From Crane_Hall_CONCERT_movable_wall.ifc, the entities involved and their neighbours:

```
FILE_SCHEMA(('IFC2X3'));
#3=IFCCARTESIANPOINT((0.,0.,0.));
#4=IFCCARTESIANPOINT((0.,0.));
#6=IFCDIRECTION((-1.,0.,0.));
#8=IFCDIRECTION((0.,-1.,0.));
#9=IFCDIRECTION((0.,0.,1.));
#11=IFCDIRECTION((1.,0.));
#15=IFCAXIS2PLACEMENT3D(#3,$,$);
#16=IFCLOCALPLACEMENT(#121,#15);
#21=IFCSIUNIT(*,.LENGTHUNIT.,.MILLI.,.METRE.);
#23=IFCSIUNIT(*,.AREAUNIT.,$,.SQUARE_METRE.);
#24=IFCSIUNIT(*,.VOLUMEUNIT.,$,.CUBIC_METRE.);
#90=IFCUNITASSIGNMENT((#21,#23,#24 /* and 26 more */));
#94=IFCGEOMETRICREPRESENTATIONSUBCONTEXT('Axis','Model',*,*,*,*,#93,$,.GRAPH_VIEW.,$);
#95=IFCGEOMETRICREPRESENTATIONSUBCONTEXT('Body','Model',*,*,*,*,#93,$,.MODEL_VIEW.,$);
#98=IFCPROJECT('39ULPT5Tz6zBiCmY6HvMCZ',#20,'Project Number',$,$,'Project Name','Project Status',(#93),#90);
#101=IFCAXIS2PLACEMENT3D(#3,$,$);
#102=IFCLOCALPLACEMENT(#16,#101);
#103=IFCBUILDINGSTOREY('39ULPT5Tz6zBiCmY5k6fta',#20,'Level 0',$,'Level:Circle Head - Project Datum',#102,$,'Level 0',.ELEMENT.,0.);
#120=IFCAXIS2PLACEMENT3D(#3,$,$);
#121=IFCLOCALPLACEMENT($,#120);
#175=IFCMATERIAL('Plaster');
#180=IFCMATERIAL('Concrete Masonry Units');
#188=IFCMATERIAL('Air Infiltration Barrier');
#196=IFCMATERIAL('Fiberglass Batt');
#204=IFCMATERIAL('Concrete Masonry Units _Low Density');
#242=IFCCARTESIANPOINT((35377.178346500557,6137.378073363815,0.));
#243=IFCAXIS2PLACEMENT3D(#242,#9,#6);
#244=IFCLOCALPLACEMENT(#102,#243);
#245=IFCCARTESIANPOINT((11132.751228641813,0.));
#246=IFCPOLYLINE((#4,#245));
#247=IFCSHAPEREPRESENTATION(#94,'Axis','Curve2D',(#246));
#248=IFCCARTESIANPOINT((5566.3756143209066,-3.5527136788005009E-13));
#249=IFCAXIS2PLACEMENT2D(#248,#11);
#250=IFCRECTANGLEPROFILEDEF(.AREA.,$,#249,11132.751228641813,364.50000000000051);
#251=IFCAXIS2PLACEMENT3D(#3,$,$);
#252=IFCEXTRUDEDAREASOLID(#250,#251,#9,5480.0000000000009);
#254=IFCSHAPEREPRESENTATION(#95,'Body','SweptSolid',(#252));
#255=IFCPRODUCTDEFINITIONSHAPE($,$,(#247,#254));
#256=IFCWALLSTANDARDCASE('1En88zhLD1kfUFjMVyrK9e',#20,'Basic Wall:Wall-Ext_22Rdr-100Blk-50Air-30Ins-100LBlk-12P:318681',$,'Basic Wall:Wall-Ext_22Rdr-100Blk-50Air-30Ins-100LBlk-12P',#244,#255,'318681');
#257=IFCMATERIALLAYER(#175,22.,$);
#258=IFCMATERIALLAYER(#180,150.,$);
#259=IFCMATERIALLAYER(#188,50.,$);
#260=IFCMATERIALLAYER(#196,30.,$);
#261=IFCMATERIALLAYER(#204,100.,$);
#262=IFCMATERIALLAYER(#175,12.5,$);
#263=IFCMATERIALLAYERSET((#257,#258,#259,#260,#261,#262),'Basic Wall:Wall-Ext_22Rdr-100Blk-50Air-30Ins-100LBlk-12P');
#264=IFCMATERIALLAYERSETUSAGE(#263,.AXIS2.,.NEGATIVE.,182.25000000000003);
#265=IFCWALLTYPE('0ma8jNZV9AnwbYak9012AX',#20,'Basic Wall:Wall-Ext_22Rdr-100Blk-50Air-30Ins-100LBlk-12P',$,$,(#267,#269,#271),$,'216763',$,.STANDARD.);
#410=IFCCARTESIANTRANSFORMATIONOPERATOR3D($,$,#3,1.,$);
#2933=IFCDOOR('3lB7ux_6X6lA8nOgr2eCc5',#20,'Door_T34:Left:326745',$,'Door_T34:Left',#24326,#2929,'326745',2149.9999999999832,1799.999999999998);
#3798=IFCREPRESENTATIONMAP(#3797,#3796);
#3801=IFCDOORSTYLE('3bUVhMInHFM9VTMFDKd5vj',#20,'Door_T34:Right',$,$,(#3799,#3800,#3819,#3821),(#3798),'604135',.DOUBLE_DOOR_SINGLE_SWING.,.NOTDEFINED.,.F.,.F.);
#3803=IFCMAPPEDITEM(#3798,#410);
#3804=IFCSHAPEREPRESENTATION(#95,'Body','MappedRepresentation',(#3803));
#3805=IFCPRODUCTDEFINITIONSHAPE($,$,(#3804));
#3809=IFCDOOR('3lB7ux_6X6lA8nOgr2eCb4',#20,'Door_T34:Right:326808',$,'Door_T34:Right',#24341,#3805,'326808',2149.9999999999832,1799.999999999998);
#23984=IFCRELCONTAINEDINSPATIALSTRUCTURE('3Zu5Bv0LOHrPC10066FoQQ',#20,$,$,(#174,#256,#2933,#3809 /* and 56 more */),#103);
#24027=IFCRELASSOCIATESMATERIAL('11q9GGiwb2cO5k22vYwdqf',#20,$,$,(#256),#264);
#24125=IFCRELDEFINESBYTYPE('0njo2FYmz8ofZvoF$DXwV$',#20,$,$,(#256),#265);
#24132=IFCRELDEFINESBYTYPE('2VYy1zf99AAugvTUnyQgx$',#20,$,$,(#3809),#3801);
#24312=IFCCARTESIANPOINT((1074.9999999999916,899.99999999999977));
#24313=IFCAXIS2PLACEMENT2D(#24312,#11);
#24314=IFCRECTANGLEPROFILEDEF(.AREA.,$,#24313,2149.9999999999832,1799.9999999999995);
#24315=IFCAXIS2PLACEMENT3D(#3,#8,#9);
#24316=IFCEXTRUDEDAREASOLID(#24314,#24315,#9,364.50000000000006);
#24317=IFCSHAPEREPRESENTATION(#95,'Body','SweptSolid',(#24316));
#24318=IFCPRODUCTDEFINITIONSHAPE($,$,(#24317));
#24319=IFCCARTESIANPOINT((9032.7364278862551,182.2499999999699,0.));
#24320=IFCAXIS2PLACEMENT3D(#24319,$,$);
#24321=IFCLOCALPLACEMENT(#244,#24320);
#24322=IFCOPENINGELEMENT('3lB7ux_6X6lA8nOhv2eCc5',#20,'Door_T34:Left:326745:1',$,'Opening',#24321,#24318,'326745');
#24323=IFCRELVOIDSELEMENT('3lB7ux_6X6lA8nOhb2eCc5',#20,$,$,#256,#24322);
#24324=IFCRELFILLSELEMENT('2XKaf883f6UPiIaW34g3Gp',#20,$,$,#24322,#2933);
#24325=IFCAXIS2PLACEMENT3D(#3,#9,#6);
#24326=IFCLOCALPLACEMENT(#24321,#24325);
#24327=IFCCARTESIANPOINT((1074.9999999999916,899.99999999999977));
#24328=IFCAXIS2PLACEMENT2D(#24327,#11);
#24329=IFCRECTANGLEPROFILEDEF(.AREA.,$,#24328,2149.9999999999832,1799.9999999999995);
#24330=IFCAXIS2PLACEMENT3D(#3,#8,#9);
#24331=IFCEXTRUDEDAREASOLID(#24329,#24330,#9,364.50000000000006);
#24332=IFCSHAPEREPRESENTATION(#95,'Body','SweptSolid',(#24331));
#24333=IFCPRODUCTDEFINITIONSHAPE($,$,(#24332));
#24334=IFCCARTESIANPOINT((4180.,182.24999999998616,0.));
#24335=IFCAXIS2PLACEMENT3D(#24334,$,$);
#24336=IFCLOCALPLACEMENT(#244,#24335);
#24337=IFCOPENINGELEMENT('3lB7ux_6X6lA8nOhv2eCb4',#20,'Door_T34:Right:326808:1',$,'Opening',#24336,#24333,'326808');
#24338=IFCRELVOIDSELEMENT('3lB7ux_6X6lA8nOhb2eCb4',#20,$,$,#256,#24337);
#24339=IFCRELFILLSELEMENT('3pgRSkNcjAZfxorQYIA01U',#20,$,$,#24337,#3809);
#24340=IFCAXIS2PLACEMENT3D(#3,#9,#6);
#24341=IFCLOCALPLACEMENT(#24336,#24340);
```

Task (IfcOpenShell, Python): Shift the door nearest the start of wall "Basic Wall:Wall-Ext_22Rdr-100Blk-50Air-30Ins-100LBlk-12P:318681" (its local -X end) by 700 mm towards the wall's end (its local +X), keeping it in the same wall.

```python
import ifcopenshell
import ifcopenshell.api.geometry
import ifcopenshell.util.placement

model = ifcopenshell.open("Crane_Hall_CONCERT_movable_wall.ifc")

door = model.by_guid("3lB7ux_6X6lA8nOgr2eCb4")
opening = door.FillsVoids[0].RelatingOpeningElement
wall = opening.VoidsElements[0].RelatingBuildingElement

wall_matrix = ifcopenshell.util.placement.get_local_placement(wall.ObjectPlacement)
shift = wall_matrix[:3, 0] * 700.0
before = ifcopenshell.util.placement.get_local_placement(door.ObjectPlacement)[:3, 3].copy()

# The door is placed relative to its opening, so it follows when the opening moves.
matrix = ifcopenshell.util.placement.get_local_placement(opening.ObjectPlacement)
matrix[:3, 3] += shift
ifcopenshell.api.geometry.edit_object_placement(
    model, product=opening, matrix=matrix, is_si=False, should_transform_children=True
)

after = ifcopenshell.util.placement.get_local_placement(door.ObjectPlacement)[:3, 3]
print("door moved by", (after - before).round(3) + 0.0)

model.write("Crane_Hall_CONCERT_movable_wall-out.ifc")
```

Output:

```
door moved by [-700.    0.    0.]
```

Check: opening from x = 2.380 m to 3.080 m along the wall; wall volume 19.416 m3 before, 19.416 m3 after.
